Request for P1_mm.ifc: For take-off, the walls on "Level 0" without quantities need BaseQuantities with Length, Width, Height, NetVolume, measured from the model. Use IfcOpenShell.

First a look at what the model holds.

```python
import ifcopenshell
import ifcopenshell.util.element
import ifcopenshell.util.unit

model = ifcopenshell.open("P1_mm.ifc")
print(model.schema)
for unit_type in ("LENGTHUNIT", "AREAUNIT", "VOLUMEUNIT"):
    print(unit_type, ifcopenshell.util.unit.calculate_unit_scale(model, unit_type))
storey = next(s for s in model.by_type("IfcBuildingStorey") if s.Name == "Level 0")
walls = [e for e in ifcopenshell.util.element.get_decomposition(storey) if e.is_a("IfcWall")]
for e in sorted(walls, key=lambda e: e.id()):
    print(e.id(), e.is_a(), e.Name, list(ifcopenshell.util.element.get_psets(e, qtos_only=True)), sep=" | ")
```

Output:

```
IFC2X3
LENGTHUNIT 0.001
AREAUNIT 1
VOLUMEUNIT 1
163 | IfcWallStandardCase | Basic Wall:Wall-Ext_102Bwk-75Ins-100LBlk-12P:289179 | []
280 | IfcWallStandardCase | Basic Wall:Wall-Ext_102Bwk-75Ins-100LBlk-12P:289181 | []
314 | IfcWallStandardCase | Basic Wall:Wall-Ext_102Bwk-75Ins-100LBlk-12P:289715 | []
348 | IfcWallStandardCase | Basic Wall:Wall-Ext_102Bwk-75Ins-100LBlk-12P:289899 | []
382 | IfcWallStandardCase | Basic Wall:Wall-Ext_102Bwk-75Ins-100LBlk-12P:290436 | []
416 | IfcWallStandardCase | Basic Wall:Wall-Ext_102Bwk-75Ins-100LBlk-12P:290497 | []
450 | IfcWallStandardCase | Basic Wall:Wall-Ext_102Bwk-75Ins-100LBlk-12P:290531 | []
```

```python
import ifcopenshell
import ifcopenshell.api.pset
import ifcopenshell.geom
import ifcopenshell.util.element
import ifcopenshell.util.shape
import ifcopenshell.util.unit

model = ifcopenshell.open("P1_mm.ifc")
unit_scale = ifcopenshell.util.unit.calculate_unit_scale(model)
volume_scale = ifcopenshell.util.unit.calculate_unit_scale(model, "VOLUMEUNIT")
settings = ifcopenshell.geom.settings()

storey = next(s for s in model.by_type("IfcBuildingStorey") if s.Name == "Level 0")
walls = [e for e in ifcopenshell.util.element.get_decomposition(storey) if e.is_a("IfcWall")]

for e in sorted(walls, key=lambda e: e.id()):
    if ifcopenshell.util.element.get_psets(e, qtos_only=True, should_inherit=False):
        continue
    # Geometry comes back in metres, in the element's own axes.
    shape = ifcopenshell.geom.create_shape(settings, e)
    values = {
        "Length": ifcopenshell.util.shape.get_x(shape.geometry) / unit_scale,
        "Width": ifcopenshell.util.shape.get_y(shape.geometry) / unit_scale,
        "Height": ifcopenshell.util.shape.get_z(shape.geometry) / unit_scale,
        "NetVolume": ifcopenshell.util.shape.get_volume(shape.geometry) / volume_scale,
    }
    qto = ifcopenshell.api.pset.add_qto(model, product=e, name="BaseQuantities")
    ifcopenshell.api.pset.edit_qto(model, qto=qto, properties=values)
    print(e.id(), {k: round(v, 3) for k, v in values.items()})

model.write("P1_mm_edited.ifc")
```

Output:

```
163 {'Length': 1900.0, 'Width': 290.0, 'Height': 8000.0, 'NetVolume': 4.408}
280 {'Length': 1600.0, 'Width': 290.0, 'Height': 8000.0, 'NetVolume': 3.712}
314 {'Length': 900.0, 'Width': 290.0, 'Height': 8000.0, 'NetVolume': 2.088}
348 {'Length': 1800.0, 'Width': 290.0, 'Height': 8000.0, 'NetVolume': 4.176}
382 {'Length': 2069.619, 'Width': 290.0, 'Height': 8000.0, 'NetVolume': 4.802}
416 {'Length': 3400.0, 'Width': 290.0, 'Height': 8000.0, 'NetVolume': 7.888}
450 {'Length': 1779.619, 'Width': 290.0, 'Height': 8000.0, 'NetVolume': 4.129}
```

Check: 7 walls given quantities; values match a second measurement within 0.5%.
